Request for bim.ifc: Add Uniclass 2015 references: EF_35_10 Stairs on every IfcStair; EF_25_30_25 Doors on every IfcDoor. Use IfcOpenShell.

First a look at what the model holds.

```python
import ifcopenshell

model = ifcopenshell.open("bim.ifc")
print(model.schema)
print("classifications:", [c.Name for c in model.by_type("IfcClassification")])
for ifc_class in ("IfcDoor", "IfcRoof", "IfcStair", "IfcWall", "IfcWindow"):
    print(ifc_class, len(model.by_type(ifc_class)))
```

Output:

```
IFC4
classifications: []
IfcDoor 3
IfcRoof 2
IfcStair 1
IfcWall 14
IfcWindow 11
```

```python
import ifcopenshell
import ifcopenshell.api.classification

model = ifcopenshell.open("bim.ifc")

system = ifcopenshell.api.classification.add_classification(model, classification="Uniclass 2015")

codes = {
    "IfcStair": ("EF_35_10", "Stairs"),
    "IfcDoor": ("EF_25_30_25", "Doors"),
}
for ifc_class, (code, name) in codes.items():
    products = model.by_type(ifc_class)
    ifcopenshell.api.classification.add_reference(
        model, products=products, classification=system, identification=code, name=name
    )
    print(code, len(products))

model.write("bim_rev.ifc")
```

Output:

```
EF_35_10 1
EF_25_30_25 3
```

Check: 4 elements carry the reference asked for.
